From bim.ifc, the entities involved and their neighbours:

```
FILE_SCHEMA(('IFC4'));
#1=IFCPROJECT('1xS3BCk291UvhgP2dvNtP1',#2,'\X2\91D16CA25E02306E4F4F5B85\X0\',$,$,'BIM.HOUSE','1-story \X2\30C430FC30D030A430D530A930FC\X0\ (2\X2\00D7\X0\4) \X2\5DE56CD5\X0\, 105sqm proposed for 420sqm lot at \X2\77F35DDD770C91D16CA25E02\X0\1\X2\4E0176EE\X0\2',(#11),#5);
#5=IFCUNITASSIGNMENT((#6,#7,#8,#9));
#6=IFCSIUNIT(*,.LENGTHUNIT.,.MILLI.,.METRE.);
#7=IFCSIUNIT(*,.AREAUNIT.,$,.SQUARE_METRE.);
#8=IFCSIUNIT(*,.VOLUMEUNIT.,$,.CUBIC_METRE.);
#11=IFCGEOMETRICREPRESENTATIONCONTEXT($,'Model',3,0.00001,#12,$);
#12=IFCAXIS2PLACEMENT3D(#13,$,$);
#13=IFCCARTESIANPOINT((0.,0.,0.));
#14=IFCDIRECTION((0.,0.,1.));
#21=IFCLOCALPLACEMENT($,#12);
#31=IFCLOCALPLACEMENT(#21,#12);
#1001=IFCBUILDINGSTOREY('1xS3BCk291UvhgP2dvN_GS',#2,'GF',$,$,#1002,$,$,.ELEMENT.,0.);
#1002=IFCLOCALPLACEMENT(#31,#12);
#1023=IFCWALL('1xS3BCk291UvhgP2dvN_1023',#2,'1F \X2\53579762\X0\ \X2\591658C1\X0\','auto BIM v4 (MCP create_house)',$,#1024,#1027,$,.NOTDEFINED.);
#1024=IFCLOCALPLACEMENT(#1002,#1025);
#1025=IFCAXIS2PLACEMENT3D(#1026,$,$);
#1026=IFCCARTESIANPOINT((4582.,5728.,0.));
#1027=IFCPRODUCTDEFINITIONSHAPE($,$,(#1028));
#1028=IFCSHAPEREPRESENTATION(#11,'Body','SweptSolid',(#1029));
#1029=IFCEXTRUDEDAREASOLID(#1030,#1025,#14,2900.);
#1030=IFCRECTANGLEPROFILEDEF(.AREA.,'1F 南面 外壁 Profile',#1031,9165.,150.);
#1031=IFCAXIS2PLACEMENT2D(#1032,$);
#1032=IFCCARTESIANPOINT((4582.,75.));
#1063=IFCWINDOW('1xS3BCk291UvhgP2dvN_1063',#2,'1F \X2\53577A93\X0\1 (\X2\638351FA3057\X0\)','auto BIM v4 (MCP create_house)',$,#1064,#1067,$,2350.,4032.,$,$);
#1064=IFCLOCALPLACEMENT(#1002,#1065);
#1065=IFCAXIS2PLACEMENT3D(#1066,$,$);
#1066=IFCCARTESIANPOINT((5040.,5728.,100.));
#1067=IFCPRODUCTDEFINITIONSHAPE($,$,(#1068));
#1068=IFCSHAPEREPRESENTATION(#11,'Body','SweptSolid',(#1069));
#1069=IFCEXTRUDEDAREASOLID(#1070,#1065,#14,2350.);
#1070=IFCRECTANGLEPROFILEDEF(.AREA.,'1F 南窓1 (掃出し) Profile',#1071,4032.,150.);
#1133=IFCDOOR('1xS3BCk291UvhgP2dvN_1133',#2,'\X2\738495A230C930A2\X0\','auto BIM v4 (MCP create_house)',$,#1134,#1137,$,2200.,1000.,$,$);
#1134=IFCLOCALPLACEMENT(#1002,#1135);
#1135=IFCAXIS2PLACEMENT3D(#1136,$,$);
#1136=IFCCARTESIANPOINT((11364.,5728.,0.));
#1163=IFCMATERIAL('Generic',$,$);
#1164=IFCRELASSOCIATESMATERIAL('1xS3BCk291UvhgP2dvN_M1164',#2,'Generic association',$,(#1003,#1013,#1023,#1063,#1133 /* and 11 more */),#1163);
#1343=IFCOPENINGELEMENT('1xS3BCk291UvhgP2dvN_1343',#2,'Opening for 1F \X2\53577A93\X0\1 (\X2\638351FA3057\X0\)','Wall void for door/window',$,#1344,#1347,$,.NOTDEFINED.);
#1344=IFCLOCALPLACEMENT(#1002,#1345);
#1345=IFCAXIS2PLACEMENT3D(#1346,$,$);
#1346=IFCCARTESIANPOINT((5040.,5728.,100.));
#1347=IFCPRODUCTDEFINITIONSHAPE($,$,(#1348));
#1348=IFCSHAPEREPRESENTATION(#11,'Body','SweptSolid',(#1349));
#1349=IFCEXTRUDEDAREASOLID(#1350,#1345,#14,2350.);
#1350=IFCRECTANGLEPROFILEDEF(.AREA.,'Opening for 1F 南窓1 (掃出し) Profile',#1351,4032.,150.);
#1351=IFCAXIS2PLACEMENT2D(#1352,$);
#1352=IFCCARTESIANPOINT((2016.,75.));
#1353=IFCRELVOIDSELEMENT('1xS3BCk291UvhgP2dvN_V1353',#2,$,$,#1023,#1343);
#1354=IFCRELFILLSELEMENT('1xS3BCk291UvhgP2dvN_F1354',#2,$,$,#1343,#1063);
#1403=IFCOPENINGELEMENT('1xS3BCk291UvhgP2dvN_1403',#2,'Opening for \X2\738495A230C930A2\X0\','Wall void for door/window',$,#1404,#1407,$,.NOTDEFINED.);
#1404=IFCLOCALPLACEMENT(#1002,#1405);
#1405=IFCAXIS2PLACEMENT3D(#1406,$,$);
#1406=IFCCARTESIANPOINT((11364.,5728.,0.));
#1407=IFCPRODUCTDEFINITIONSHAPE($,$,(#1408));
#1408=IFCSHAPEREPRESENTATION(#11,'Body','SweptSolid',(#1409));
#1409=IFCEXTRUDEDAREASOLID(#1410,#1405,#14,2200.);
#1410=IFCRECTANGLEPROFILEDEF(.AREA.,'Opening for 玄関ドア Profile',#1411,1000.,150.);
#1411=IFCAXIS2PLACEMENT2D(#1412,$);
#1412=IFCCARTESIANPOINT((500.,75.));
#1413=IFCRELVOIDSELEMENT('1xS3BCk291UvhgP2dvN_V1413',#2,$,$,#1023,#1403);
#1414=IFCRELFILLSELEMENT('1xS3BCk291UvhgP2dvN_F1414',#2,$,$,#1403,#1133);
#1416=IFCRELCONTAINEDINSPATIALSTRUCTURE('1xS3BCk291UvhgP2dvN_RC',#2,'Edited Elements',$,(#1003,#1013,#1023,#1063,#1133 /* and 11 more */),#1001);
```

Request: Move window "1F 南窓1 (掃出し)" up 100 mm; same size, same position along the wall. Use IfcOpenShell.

```python
import numpy as np
import ifcopenshell
import ifcopenshell.api.geometry
import ifcopenshell.util.placement
import ifcopenshell.util.unit

model = ifcopenshell.open("bim.ifc")
unit_scale = ifcopenshell.util.unit.calculate_unit_scale(model)

window = model.by_id(1063)
opening = window.FillsVoids[0].RelatingOpeningElement
dz = 0.1 / unit_scale

shift = np.array([0.0, 0.0, dz])
# The window is not placed relative to its opening, so move both.
for product in (opening, window):
    matrix = ifcopenshell.util.placement.get_local_placement(product.ObjectPlacement)
    matrix[:3, 3] += shift
    ifcopenshell.api.geometry.edit_object_placement(model, product=product, matrix=matrix, is_si=False)

print(f"moved by {dz * unit_scale:+.3f} m")

model.write("bim-out.ifc")
```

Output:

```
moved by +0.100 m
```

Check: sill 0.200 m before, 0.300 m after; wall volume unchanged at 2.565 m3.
